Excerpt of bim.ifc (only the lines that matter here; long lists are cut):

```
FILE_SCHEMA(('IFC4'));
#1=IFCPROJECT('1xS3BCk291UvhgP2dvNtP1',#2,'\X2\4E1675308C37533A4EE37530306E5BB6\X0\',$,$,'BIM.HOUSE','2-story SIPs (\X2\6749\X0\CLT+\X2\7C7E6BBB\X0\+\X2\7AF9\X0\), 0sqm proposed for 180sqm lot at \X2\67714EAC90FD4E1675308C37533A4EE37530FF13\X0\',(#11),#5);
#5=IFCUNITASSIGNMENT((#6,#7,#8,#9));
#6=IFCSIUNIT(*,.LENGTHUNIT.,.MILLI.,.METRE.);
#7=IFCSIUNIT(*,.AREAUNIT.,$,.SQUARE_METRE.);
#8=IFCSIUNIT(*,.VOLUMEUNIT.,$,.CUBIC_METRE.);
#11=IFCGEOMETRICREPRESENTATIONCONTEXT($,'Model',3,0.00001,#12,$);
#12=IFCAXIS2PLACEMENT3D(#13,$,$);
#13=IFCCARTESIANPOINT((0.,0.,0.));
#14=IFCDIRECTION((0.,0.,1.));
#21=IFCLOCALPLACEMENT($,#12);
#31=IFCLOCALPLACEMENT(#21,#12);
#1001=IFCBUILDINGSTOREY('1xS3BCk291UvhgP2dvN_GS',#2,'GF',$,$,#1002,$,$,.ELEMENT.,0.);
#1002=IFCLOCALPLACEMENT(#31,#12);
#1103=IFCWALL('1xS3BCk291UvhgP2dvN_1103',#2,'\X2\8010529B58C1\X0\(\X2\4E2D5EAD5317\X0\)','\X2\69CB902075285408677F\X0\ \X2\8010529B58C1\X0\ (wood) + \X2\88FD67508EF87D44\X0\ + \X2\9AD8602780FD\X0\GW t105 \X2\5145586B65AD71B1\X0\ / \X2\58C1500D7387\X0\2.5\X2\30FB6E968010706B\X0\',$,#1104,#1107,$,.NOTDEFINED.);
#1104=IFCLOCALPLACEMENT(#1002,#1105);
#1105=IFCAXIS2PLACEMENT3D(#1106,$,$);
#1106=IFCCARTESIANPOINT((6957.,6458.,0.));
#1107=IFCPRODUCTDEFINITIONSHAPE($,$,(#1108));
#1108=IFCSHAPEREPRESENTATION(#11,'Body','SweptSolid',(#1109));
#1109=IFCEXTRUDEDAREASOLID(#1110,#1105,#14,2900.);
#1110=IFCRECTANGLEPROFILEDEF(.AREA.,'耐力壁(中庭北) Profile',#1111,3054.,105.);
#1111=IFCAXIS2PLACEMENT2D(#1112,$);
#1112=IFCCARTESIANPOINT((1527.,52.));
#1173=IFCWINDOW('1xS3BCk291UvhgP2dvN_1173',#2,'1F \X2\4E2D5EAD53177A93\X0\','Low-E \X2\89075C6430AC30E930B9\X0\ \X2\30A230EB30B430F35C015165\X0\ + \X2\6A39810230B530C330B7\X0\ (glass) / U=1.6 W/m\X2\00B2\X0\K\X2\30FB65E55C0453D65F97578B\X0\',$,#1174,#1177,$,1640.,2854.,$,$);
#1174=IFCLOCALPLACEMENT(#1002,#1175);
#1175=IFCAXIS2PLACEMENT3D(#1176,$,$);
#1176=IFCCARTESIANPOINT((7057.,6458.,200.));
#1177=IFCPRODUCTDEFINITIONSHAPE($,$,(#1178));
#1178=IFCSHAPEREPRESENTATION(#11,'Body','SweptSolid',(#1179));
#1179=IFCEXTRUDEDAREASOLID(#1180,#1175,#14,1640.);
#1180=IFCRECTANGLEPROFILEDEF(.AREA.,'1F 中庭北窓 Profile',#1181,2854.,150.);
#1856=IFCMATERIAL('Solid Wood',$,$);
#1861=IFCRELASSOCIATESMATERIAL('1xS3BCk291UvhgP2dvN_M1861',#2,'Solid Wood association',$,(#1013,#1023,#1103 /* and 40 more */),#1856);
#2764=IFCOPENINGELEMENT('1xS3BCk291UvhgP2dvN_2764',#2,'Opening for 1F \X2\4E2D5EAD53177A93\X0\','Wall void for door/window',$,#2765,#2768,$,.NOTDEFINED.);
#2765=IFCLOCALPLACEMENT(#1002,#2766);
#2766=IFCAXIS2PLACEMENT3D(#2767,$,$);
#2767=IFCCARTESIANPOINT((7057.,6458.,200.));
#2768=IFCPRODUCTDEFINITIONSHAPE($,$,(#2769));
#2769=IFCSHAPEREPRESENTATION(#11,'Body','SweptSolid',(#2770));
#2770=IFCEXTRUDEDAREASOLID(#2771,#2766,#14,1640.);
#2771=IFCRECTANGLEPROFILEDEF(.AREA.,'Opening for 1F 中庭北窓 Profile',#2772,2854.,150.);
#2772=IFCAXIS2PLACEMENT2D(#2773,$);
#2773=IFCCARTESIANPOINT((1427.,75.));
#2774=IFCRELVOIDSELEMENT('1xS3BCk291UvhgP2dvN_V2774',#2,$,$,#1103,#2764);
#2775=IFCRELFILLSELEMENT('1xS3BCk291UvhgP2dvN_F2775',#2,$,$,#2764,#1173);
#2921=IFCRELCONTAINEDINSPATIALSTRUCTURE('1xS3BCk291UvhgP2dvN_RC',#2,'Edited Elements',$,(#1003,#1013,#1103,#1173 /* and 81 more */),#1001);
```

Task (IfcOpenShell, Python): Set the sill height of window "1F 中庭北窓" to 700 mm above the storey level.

```python
import numpy as np
import ifcopenshell
import ifcopenshell.api.geometry
import ifcopenshell.geom
import ifcopenshell.util.element
import ifcopenshell.util.placement
import ifcopenshell.util.shape
import ifcopenshell.util.unit

model = ifcopenshell.open("bim.ifc")
unit_scale = ifcopenshell.util.unit.calculate_unit_scale(model)

window = model.by_guid("1xS3BCk291UvhgP2dvN_1173")
opening = window.FillsVoids[0].RelatingOpeningElement
storey = ifcopenshell.util.element.get_container(window, ifc_class="IfcBuildingStorey")
level = ifcopenshell.util.placement.get_local_placement(storey.ObjectPlacement)[2, 3]

# The opening's origin need not be at the sill, so measure its lowest point.
shape = ifcopenshell.geom.create_shape(ifcopenshell.geom.settings(), opening)
bottom = ifcopenshell.util.shape.get_shape_bottom_elevation(shape, shape.geometry) / unit_scale
dz = level + 0.7 / unit_scale - bottom

shift = np.array([0.0, 0.0, dz])
# The window is not placed relative to its opening, so move both.
for product in (opening, window):
    matrix = ifcopenshell.util.placement.get_local_placement(product.ObjectPlacement)
    matrix[:3, 3] += shift
    ifcopenshell.api.geometry.edit_object_placement(model, product=product, matrix=matrix, is_si=False)

print(f"moved by {dz * unit_scale:+.3f} m")

model.write("bim-out.ifc")
```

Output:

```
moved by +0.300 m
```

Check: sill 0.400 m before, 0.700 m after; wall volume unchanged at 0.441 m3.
